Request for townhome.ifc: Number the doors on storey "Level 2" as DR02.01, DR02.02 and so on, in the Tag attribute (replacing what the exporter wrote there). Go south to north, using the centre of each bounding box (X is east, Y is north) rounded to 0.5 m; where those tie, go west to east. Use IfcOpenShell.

First a look at what the model holds.

```python
import ifcopenshell
import ifcopenshell.util.element
import ifcopenshell.util.placement

model = ifcopenshell.open("townhome.ifc")
print(model.schema)
storey = next(s for s in model.by_type("IfcBuildingStorey") if s.Name == "Level 2")
doors = [e for e in ifcopenshell.util.element.get_decomposition(storey) if e.is_a("IfcDoor")]
for e in sorted(doors, key=lambda e: e.id()):
    origin = ifcopenshell.util.placement.get_local_placement(e.ObjectPlacement)[:3, 3]
    print(e.id(), e.Tag, e.Name, origin.round(2) + 0.0, sep=" | ")
```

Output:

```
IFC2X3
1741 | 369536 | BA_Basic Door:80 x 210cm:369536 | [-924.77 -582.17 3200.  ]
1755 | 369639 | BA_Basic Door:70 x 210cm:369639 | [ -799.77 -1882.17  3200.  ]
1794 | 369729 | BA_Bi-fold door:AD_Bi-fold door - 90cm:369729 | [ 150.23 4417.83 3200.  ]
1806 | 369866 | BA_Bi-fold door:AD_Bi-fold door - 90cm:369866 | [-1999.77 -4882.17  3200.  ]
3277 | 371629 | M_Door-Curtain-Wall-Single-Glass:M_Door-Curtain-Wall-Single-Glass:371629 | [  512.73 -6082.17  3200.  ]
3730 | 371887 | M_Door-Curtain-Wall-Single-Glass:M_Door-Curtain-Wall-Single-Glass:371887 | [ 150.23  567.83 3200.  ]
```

```python
import ifcopenshell
import ifcopenshell.geom
import ifcopenshell.util.element
import ifcopenshell.util.shape

model = ifcopenshell.open("townhome.ifc")
settings = ifcopenshell.geom.settings()
settings.set("use-world-coords", True)


def centre(element):
    shape = ifcopenshell.geom.create_shape(settings, element)
    return ifcopenshell.util.shape.get_bbox_centroid(shape.geometry)


storey = next(s for s in model.by_type("IfcBuildingStorey") if s.Name == "Level 2")
doors = [e for e in ifcopenshell.util.element.get_decomposition(storey) if e.is_a("IfcDoor")]

# Insertion points can sit at a corner or the storey origin, so sort by the geometry (in metres).
centres = {e: centre(e) for e in doors}
doors.sort(key=lambda e: (round(centres[e][1] / 0.5), centres[e][0]))

for i, e in enumerate(doors, start=1):
    number = f"DR02.{i:02d}"
    e.Tag = number
    print(e.id(), number)

model.write("townhome_v2.ifc")
```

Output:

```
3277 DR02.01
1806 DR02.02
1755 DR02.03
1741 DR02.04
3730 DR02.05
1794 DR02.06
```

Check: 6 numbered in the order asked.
